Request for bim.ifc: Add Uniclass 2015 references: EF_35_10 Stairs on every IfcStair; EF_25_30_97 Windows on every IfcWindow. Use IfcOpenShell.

First a look at what the model holds.

```python
import ifcopenshell

model = ifcopenshell.open("bim.ifc")
print(model.schema)
print("classifications:", [c.Name for c in model.by_type("IfcClassification")])
for ifc_class in ("IfcDoor", "IfcRoof", "IfcStair", "IfcWall", "IfcWindow"):
    print(ifc_class, len(model.by_type(ifc_class)))
```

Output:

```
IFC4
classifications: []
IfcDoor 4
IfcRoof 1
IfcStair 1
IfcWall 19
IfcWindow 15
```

```python
import ifcopenshell
import ifcopenshell.api.classification

model = ifcopenshell.open("bim.ifc")

system = ifcopenshell.api.classification.add_classification(model, classification="Uniclass 2015")

codes = {
    "IfcStair": ("EF_35_10", "Stairs"),
    "IfcWindow": ("EF_25_30_97", "Windows"),
}
for ifc_class, (code, name) in codes.items():
    products = model.by_type(ifc_class)
    ifcopenshell.api.classification.add_reference(
        model, products=products, classification=system, identification=code, name=name
    )
    print(code, len(products))

model.write("bim_rev.ifc")
```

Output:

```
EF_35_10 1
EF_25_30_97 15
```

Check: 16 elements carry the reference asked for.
